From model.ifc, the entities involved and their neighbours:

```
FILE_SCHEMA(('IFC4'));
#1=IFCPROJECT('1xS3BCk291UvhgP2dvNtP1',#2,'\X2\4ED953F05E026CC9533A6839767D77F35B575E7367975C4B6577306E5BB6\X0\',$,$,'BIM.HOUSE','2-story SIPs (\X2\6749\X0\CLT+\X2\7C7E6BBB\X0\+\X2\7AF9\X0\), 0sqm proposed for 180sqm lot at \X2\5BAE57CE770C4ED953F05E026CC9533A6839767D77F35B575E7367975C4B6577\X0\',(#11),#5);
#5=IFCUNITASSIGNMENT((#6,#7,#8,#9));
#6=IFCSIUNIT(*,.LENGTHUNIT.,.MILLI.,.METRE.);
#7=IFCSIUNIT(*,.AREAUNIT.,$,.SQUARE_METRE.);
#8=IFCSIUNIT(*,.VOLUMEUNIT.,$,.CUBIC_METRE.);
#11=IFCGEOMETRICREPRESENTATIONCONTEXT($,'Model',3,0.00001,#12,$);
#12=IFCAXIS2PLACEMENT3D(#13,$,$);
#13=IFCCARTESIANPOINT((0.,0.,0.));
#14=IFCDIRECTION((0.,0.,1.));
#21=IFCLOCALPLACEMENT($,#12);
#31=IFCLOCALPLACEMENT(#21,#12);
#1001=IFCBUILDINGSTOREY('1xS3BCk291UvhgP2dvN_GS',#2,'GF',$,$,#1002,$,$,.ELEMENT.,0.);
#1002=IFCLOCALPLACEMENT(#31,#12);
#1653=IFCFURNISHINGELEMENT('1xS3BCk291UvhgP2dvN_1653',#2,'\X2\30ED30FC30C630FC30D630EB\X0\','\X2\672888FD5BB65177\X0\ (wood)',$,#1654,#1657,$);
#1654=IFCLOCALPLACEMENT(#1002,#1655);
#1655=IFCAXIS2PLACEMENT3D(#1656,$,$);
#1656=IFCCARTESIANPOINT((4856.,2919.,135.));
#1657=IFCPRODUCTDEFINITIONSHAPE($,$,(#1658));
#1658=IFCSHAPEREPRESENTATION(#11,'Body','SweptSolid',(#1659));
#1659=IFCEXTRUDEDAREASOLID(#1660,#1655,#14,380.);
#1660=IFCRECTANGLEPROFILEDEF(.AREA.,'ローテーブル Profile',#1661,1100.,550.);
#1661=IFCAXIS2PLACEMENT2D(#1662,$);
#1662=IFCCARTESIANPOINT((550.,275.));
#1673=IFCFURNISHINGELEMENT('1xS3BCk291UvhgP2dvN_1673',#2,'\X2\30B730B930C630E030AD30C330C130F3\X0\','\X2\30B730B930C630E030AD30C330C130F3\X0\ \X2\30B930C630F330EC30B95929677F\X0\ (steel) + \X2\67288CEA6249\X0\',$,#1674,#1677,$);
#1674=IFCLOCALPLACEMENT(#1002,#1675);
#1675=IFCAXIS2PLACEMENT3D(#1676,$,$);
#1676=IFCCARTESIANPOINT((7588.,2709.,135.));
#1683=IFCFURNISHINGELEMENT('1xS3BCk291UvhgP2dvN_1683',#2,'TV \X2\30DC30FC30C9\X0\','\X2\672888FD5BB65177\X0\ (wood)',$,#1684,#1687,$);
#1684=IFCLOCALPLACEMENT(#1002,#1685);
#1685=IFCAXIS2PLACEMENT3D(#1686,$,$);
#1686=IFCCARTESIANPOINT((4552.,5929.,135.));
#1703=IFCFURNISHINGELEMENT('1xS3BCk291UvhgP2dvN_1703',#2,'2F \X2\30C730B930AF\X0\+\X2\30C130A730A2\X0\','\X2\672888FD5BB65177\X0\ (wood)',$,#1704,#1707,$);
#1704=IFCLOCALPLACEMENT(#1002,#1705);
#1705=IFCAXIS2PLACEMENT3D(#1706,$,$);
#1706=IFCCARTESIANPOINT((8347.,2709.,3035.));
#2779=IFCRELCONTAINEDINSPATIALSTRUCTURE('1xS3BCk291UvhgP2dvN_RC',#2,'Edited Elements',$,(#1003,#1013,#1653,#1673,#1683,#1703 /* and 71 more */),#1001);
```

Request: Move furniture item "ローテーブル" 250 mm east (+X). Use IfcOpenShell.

```python
import ifcopenshell
import ifcopenshell.api.geometry
import ifcopenshell.util.placement
import ifcopenshell.util.unit

model = ifcopenshell.open("model.ifc")
unit_scale = ifcopenshell.util.unit.calculate_unit_scale(model)

item = model.by_guid("1xS3BCk291UvhgP2dvN_1653")
matrix = ifcopenshell.util.placement.get_local_placement(item.ObjectPlacement)
matrix[0, 3] += 0.25 / unit_scale
ifcopenshell.api.geometry.edit_object_placement(model, product=item, matrix=matrix, is_si=False)

print(ifcopenshell.util.placement.get_local_placement(item.ObjectPlacement).round(3) + 0.0)

model.write("model_updated.ifc")
```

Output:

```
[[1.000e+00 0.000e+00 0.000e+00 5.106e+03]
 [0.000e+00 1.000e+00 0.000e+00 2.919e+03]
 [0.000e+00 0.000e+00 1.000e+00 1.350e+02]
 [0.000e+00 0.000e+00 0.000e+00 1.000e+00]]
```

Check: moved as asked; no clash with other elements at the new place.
